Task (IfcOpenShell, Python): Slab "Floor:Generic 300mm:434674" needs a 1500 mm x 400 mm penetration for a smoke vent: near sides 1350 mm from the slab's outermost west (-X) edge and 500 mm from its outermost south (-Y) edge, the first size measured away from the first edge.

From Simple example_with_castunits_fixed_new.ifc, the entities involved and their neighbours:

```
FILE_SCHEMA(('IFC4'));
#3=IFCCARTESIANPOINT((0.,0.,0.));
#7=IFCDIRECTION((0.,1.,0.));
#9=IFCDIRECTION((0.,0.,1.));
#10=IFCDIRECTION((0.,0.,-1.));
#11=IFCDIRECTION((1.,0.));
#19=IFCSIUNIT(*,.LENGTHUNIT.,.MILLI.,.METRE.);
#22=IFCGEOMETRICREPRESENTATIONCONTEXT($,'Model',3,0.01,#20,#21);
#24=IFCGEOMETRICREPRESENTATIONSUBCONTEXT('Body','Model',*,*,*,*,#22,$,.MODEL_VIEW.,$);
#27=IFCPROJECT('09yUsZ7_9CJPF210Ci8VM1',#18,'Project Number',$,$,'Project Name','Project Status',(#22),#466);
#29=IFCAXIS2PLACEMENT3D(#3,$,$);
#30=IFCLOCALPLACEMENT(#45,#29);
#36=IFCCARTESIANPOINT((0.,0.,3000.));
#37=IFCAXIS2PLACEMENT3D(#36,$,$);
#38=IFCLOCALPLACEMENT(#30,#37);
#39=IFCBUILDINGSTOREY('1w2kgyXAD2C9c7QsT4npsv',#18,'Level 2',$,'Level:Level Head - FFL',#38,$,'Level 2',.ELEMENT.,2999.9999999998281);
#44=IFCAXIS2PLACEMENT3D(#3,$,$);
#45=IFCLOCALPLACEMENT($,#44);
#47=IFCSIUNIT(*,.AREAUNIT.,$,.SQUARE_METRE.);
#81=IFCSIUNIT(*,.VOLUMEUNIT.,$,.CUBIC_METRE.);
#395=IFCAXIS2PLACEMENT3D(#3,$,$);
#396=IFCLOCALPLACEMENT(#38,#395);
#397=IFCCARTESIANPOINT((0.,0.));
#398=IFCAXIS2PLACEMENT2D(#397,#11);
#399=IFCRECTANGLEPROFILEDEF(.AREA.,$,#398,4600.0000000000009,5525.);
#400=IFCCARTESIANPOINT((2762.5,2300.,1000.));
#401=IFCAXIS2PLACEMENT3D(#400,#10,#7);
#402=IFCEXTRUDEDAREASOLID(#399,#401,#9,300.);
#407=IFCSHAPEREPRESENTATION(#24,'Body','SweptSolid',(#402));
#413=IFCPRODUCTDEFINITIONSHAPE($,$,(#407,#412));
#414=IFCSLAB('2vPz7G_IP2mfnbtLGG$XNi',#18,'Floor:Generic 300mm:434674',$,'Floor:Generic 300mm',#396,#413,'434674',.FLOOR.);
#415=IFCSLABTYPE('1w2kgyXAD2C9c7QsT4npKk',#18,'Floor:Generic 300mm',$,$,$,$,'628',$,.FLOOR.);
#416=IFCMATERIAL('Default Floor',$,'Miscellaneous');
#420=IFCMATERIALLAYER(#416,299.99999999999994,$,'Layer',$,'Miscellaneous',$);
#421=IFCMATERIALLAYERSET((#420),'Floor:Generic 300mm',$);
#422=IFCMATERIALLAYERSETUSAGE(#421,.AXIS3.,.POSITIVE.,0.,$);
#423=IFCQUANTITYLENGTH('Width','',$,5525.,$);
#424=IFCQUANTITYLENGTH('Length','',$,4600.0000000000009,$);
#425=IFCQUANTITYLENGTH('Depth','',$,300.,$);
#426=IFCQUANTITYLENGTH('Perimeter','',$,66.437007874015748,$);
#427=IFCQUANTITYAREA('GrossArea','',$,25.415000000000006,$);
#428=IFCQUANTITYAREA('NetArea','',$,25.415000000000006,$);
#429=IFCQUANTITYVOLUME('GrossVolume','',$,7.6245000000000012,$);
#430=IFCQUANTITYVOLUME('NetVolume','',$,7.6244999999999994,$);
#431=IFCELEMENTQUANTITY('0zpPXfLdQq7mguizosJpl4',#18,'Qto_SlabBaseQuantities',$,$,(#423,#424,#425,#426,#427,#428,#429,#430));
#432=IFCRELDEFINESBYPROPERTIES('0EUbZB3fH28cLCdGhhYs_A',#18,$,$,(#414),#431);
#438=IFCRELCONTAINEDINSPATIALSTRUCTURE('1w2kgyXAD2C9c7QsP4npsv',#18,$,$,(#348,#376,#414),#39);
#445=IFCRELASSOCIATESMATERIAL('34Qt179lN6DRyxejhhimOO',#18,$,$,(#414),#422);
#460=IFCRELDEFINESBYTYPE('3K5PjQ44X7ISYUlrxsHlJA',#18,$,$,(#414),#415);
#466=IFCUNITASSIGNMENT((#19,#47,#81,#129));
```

```python
import numpy as np
import ifcopenshell
import ifcopenshell.api.feature
import ifcopenshell.api.geometry
import ifcopenshell.api.pset
import ifcopenshell.api.root
import ifcopenshell.geom
import ifcopenshell.util.element
import ifcopenshell.util.placement
import ifcopenshell.util.representation
import ifcopenshell.util.shape
import ifcopenshell.util.unit

model = ifcopenshell.open("Simple example_with_castunits_fixed_new.ifc")
unit_scale = ifcopenshell.util.unit.calculate_unit_scale(model)
area_scale = ifcopenshell.util.unit.calculate_unit_scale(model, "AREAUNIT")
volume_scale = ifcopenshell.util.unit.calculate_unit_scale(model, "VOLUMEUNIT")
settings = ifcopenshell.geom.settings()


def volume(element):
    """Net volume in cubic metres, openings subtracted."""
    shape = ifcopenshell.geom.create_shape(settings, element)
    return ifcopenshell.util.shape.get_volume(shape.geometry)


slab = model.by_id(414)
before = volume(slab)

# Extent in the slab's own axes, in metres. The edges named are its -X and -Y sides.
slab_shape = ifcopenshell.geom.create_shape(settings, slab)
vertices = ifcopenshell.util.shape.get_vertices(slab_shape.geometry)
x_min, y_min, bottom = vertices.min(axis=0)
top = vertices[:, 2].max()

opening = ifcopenshell.api.root.create_entity(model, ifc_class="IfcOpeningElement", name="Smoke vent opening", predefined_type="OPENING")
context = ifcopenshell.util.representation.get_context(model, "Model", "Body", "MODEL_VIEW")
width, depth = 1.5, 0.4
outline = [(0.0, 0.0), (width, 0.0), (width, depth), (0.0, depth), (0.0, 0.0)]
# Overshoot both faces by 50 mm so the cut is clean.
shape = ifcopenshell.api.geometry.add_slab_representation(
    model, context=context, depth=top - bottom + 0.1, polyline=outline
)
ifcopenshell.api.geometry.assign_representation(model, product=opening, representation=shape)

matrix = ifcopenshell.util.placement.get_local_placement(slab.ObjectPlacement)
matrix[:, 3] = matrix @ np.append(np.array([x_min + 1.35, y_min + 0.5, bottom - 0.05]) / unit_scale, 1.0)
ifcopenshell.api.geometry.edit_object_placement(model, product=opening, matrix=matrix, is_si=False)
ifcopenshell.api.feature.add_feature(model, feature=opening, element=slab)

after = volume(slab)

# Update the slab's stored quantities.
qto = model.by_id(ifcopenshell.util.element.get_pset(slab, "Qto_SlabBaseQuantities", should_inherit=False)["id"])
ifcopenshell.api.pset.edit_qto(model, qto=qto, properties={
    "NetArea": after / (top - bottom) / area_scale,
    "NetVolume": after / volume_scale,
})

print(f"slab volume {before:.3f} -> {after:.3f} m3")

model.write("Simple example_with_castunits_fixed_new_updated.ifc")
```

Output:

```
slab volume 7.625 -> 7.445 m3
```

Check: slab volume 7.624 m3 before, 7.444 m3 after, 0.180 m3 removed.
